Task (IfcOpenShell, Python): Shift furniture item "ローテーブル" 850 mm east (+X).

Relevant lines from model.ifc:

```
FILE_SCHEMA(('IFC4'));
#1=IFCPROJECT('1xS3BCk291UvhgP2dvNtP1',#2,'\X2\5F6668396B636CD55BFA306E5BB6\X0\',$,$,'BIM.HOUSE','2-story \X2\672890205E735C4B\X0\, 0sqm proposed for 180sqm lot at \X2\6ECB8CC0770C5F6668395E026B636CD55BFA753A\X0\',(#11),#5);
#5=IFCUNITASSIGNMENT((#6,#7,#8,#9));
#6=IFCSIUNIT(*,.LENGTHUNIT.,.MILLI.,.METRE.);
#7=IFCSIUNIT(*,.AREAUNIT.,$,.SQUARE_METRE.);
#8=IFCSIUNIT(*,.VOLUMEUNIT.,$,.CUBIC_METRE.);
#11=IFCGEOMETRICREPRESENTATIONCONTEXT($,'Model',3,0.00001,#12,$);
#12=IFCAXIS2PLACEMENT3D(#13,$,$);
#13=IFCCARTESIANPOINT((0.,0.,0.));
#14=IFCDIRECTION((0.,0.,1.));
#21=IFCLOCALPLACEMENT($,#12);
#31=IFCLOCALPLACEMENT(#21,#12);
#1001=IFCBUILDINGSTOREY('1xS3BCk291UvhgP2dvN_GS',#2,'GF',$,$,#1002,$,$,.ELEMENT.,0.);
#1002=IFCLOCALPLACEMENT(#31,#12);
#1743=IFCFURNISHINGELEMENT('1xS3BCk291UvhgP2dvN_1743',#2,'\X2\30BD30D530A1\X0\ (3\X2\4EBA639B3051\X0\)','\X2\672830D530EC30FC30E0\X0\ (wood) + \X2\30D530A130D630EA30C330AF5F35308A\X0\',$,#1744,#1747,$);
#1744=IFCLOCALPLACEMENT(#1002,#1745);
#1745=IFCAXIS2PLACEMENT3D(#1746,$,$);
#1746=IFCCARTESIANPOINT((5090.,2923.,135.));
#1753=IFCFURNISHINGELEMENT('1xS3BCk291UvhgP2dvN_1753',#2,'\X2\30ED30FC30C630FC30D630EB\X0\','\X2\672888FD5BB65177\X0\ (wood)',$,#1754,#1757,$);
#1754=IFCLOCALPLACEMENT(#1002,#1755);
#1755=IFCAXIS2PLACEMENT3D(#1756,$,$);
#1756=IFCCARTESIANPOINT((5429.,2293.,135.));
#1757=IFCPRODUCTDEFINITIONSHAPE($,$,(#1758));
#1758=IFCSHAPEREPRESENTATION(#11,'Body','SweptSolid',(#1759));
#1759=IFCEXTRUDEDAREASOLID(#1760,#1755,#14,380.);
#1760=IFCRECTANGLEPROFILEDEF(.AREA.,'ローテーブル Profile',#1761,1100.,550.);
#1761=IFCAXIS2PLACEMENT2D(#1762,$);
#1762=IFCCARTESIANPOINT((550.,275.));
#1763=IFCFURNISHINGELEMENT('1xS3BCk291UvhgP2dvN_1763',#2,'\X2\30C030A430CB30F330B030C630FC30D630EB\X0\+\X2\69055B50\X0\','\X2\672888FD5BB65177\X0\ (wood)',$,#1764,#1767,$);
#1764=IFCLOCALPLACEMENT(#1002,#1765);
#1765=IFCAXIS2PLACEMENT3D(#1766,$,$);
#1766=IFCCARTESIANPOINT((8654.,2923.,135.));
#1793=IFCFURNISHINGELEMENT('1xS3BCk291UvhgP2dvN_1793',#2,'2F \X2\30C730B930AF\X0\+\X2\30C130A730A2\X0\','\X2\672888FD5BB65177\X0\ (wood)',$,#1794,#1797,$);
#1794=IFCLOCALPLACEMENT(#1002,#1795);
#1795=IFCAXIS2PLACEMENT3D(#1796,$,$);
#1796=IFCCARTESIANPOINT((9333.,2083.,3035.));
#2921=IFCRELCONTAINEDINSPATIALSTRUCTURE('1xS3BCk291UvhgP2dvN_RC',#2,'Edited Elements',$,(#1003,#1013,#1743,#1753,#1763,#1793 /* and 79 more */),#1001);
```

```python
import ifcopenshell
import ifcopenshell.api.geometry
import ifcopenshell.util.placement

model = ifcopenshell.open("model.ifc")

item = model.by_guid("1xS3BCk291UvhgP2dvN_1753")
matrix = ifcopenshell.util.placement.get_local_placement(item.ObjectPlacement)
matrix[0, 3] += 850.0
ifcopenshell.api.geometry.edit_object_placement(model, product=item, matrix=matrix, is_si=False)

print(ifcopenshell.util.placement.get_local_placement(item.ObjectPlacement).round(3) + 0.0)

model.write("model_rev.ifc")
```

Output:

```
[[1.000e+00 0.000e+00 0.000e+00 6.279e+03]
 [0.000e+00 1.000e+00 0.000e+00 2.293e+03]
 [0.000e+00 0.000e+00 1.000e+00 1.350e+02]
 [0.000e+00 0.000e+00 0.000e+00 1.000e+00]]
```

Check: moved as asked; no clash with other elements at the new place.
